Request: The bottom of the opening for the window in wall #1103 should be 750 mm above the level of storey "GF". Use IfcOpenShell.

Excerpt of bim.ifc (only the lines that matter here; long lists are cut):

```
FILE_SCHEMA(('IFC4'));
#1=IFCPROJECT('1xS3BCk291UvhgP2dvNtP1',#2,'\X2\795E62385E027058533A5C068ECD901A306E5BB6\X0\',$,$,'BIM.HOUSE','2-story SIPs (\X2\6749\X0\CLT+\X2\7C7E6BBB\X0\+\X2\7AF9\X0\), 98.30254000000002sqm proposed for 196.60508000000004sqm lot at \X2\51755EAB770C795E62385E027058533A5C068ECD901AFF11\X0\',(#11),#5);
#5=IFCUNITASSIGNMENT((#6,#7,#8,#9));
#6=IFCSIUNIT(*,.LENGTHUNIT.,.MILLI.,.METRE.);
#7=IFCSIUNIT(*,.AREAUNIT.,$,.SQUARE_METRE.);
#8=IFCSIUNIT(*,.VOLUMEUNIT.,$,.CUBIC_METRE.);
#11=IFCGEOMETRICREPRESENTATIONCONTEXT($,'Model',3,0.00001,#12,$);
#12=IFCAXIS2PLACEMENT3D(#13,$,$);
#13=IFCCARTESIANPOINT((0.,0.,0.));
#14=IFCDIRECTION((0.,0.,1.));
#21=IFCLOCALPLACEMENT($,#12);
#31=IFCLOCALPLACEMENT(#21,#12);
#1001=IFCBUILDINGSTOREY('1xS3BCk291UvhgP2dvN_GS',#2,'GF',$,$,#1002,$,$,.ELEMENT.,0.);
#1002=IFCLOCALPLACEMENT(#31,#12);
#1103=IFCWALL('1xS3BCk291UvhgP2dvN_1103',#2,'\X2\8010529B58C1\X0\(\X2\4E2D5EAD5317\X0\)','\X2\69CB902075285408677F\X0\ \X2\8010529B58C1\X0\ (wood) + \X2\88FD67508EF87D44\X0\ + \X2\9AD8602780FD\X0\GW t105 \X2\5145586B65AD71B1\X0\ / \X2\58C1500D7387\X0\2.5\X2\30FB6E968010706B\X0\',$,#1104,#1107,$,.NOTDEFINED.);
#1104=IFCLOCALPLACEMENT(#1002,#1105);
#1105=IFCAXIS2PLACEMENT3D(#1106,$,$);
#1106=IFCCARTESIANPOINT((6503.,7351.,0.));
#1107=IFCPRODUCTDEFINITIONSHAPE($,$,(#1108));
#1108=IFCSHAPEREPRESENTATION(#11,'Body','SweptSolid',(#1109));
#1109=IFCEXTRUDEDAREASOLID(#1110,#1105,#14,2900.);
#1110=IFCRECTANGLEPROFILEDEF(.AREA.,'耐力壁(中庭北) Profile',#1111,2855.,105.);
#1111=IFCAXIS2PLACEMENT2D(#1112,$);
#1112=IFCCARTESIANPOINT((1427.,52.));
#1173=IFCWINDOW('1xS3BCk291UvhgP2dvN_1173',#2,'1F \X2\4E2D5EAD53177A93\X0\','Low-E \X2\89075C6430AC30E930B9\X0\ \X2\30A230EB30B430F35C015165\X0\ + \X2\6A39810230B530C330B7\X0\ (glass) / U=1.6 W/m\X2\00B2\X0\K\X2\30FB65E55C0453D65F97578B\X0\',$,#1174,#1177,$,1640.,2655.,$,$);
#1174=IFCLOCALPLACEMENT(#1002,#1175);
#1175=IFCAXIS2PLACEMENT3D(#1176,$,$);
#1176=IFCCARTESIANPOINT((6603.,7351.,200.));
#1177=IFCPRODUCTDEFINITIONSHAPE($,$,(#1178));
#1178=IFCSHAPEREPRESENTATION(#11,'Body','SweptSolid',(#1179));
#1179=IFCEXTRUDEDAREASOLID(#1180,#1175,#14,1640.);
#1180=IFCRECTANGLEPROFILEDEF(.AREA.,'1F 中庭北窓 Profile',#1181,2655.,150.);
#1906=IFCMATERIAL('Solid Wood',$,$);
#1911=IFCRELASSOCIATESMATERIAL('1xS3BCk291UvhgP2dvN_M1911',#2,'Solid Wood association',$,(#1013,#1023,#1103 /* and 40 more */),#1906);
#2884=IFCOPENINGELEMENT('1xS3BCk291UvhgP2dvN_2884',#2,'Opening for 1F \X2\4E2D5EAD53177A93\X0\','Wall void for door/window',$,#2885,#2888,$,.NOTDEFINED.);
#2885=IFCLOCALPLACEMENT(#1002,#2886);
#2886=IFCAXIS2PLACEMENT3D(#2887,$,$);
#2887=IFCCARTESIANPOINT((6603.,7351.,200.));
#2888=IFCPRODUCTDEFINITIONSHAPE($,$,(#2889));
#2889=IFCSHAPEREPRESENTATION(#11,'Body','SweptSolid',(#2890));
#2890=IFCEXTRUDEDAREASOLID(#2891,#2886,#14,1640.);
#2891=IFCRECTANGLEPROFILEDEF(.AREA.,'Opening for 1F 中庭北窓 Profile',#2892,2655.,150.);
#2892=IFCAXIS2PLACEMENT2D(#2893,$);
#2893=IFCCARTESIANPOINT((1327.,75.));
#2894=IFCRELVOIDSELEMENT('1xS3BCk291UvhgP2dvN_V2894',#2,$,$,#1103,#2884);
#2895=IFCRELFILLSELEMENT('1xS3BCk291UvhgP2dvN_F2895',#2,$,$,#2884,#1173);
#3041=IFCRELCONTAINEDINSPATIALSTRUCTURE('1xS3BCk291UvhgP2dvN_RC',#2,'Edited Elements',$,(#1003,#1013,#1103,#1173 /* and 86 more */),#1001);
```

```python
import numpy as np
import ifcopenshell
import ifcopenshell.api.geometry
import ifcopenshell.geom
import ifcopenshell.util.element
import ifcopenshell.util.placement
import ifcopenshell.util.shape
import ifcopenshell.util.unit

model = ifcopenshell.open("bim.ifc")
unit_scale = ifcopenshell.util.unit.calculate_unit_scale(model)

window = model.by_guid("1xS3BCk291UvhgP2dvN_1173")
opening = window.FillsVoids[0].RelatingOpeningElement
storey = ifcopenshell.util.element.get_container(window, ifc_class="IfcBuildingStorey")
level = ifcopenshell.util.placement.get_local_placement(storey.ObjectPlacement)[2, 3]

# The opening's origin need not be at the sill, so measure its lowest point.
shape = ifcopenshell.geom.create_shape(ifcopenshell.geom.settings(), opening)
bottom = ifcopenshell.util.shape.get_shape_bottom_elevation(shape, shape.geometry) / unit_scale
dz = level + 0.75 / unit_scale - bottom

shift = np.array([0.0, 0.0, dz])
# The window is not placed relative to its opening, so move both.
for product in (opening, window):
    matrix = ifcopenshell.util.placement.get_local_placement(product.ObjectPlacement)
    matrix[:3, 3] += shift
    ifcopenshell.api.geometry.edit_object_placement(model, product=product, matrix=matrix, is_si=False)

print(f"moved by {dz * unit_scale:+.3f} m")

model.write("bim_updated.ifc")
```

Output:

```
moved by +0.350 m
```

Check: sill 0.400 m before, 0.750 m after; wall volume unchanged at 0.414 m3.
